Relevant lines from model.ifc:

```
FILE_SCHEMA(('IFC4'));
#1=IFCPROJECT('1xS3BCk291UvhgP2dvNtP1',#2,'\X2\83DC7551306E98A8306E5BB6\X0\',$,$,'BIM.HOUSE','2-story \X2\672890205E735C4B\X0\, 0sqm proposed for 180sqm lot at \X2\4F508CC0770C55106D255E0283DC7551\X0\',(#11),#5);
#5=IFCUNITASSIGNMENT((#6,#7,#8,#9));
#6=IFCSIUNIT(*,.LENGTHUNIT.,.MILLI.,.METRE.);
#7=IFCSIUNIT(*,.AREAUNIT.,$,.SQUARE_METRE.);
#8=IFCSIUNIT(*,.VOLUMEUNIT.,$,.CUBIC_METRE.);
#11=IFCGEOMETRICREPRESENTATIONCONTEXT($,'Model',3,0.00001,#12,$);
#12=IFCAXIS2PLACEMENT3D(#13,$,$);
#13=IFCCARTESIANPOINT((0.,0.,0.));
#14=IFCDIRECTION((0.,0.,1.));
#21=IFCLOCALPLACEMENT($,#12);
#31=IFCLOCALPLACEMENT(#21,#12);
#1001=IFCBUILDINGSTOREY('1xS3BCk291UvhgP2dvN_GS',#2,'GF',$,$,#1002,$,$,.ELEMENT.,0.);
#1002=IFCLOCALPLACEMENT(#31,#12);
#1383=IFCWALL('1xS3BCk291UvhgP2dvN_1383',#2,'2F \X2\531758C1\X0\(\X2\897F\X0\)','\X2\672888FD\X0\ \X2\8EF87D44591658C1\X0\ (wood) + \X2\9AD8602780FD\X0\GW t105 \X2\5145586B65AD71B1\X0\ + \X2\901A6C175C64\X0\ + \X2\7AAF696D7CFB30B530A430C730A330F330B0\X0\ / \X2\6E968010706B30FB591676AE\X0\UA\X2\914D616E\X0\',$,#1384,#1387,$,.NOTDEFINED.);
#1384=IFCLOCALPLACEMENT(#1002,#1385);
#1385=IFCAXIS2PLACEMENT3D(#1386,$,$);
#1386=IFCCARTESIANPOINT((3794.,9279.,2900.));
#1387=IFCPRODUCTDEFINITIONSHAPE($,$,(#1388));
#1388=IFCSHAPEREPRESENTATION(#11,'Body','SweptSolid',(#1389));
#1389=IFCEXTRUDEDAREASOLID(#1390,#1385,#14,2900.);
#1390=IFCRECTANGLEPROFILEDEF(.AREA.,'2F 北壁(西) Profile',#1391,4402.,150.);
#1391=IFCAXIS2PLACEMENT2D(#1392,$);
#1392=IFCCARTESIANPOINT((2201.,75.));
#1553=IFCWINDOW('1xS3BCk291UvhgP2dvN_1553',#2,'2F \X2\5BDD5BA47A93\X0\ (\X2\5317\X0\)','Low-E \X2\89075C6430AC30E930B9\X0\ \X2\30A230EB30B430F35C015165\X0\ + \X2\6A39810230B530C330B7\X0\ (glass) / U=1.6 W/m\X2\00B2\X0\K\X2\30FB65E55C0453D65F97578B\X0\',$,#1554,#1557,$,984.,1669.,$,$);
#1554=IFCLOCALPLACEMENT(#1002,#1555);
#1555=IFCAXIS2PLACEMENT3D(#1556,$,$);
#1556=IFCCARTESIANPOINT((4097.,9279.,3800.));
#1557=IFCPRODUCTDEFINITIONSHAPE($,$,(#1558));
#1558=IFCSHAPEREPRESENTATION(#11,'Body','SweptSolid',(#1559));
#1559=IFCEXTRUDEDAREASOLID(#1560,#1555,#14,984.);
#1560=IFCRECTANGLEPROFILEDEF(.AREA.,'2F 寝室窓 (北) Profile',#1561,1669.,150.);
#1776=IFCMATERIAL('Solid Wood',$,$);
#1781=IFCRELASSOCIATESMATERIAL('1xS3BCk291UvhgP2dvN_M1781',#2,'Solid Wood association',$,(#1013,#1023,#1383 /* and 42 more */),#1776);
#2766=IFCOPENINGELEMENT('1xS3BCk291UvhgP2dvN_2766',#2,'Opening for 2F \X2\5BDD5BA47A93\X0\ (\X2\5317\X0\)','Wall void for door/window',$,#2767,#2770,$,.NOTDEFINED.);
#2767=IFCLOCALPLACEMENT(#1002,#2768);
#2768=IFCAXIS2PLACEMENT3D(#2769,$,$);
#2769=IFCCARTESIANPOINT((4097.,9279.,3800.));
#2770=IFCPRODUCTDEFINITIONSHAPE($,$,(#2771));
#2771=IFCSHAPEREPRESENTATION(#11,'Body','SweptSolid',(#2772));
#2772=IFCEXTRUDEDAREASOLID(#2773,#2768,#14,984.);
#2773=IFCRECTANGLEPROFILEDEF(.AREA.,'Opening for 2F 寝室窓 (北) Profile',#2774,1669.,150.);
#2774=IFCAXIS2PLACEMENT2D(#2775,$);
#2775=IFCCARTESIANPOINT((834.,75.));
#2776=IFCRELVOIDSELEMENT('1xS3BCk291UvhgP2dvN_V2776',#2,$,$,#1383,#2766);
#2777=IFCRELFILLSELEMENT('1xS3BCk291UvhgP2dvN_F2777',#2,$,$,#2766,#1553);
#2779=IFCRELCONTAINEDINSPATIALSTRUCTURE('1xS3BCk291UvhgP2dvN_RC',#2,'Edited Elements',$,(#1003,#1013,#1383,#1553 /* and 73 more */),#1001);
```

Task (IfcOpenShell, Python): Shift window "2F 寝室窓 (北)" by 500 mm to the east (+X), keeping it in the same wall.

```python
import ifcopenshell
import ifcopenshell.api.geometry
import ifcopenshell.util.placement
import ifcopenshell.util.unit

model = ifcopenshell.open("model.ifc")
unit_scale = ifcopenshell.util.unit.calculate_unit_scale(model)

window = model.by_guid("1xS3BCk291UvhgP2dvN_1553")
opening = window.FillsVoids[0].RelatingOpeningElement
wall = opening.VoidsElements[0].RelatingBuildingElement

wall_matrix = ifcopenshell.util.placement.get_local_placement(wall.ObjectPlacement)
shift = wall_matrix[:3, 0] * 0.5 / unit_scale
before = ifcopenshell.util.placement.get_local_placement(window.ObjectPlacement)[:3, 3].copy()

# The window is not placed relative to its opening, so move both.
for product in (opening, window):
    matrix = ifcopenshell.util.placement.get_local_placement(product.ObjectPlacement)
    matrix[:3, 3] += shift
    ifcopenshell.api.geometry.edit_object_placement(model, product=product, matrix=matrix, is_si=False)

after = ifcopenshell.util.placement.get_local_placement(window.ObjectPlacement)[:3, 3]
print("window moved by", (after - before).round(3) + 0.0)

model.write("model_rev.ifc")
```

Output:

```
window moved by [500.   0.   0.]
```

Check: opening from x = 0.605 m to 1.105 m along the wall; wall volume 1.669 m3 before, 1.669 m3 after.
